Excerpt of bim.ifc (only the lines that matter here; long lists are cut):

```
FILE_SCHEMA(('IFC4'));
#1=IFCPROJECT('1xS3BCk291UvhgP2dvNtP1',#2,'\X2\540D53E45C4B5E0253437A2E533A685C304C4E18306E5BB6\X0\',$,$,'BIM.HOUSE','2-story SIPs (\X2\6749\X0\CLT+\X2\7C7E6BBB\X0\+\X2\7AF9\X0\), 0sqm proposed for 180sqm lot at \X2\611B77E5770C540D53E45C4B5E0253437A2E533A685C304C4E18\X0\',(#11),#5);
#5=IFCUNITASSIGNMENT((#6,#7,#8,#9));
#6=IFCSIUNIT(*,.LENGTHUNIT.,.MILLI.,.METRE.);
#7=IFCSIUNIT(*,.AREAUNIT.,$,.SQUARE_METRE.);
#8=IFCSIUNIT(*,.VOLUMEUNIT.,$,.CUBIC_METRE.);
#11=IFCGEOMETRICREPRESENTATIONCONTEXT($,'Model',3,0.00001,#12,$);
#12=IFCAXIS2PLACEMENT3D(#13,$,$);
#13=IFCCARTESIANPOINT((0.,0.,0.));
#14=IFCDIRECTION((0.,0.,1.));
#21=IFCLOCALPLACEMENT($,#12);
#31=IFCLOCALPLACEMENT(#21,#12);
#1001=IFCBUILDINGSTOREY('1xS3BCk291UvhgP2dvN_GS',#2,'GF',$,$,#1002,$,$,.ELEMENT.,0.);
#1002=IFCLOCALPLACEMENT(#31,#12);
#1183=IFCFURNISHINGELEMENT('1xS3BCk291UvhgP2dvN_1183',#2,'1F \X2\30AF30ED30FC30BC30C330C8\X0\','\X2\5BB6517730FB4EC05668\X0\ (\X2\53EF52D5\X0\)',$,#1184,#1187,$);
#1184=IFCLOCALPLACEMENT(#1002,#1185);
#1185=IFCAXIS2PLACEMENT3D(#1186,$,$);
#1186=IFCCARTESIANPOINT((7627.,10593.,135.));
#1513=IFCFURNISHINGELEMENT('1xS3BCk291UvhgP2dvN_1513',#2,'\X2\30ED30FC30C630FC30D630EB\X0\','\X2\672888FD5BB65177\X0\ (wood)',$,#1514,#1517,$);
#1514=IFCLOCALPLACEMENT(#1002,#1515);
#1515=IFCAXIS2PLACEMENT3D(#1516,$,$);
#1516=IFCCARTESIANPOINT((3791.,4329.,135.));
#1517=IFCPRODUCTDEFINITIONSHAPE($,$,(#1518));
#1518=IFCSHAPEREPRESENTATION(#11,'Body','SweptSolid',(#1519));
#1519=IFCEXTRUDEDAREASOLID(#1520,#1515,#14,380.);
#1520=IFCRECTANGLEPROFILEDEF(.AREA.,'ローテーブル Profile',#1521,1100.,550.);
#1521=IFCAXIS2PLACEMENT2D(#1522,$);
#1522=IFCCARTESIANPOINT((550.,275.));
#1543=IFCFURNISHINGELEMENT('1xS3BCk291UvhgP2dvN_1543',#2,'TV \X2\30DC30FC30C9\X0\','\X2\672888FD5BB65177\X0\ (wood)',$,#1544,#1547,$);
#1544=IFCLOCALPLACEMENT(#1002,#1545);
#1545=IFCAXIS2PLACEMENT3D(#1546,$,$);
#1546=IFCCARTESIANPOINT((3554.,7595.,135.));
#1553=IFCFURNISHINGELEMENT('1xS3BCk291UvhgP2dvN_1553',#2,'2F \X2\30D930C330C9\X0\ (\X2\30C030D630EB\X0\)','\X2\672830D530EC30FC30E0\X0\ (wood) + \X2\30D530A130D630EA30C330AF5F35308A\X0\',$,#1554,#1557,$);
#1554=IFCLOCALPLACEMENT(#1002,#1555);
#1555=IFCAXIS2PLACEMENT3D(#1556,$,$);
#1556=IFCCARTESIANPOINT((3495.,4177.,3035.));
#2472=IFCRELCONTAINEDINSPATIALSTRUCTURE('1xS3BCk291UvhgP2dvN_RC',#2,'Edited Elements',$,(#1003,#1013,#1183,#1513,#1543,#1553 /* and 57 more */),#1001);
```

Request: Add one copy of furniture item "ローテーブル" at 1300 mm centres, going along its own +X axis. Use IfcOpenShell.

```python
import ifcopenshell
import ifcopenshell.api.geometry
import ifcopenshell.api.root
import ifcopenshell.util.element
import ifcopenshell.util.placement

model = ifcopenshell.open("bim.ifc")


def reuse_history(source, copy):
    """copy_class also copies each property set's owner history, people and application; keep the originals."""
    for rel in copy.IsDefinedBy:
        if rel.is_a("IfcRelDefinesByProperties") and (history := rel.RelatingPropertyDefinition.OwnerHistory):
            rel.RelatingPropertyDefinition.OwnerHistory = source.OwnerHistory
            ifcopenshell.util.element.remove_deep2(model, history)


source = model.by_id(1513)
base = ifcopenshell.util.placement.get_local_placement(source.ObjectPlacement)
step = base[:3, 0] * 1300.0

for i in range(1, 2):
    copy = ifcopenshell.api.root.copy_class(model, product=source)
    copy.Representation = ifcopenshell.util.element.copy_deep(
        model, source.Representation, exclude=["IfcGeometricRepresentationContext", "IfcRepresentationMap"]
    )
    reuse_history(source, copy)
    matrix = base.copy()
    matrix[:3, 3] += i * step
    print("added at", matrix[:3, 3].round(3) + 0.0)
    ifcopenshell.api.geometry.edit_object_placement(model, product=copy, matrix=matrix, is_si=False)

model.write("bim_updated.ifc")
```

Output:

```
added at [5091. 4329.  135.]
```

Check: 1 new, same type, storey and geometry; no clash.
